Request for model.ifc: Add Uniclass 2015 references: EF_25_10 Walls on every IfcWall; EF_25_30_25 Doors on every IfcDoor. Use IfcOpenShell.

First a look at what the model holds.

```python
import ifcopenshell

model = ifcopenshell.open("model.ifc")
print(model.schema)
print("classifications:", [c.Name for c in model.by_type("IfcClassification")])
for ifc_class in ("IfcDoor", "IfcRoof", "IfcStair", "IfcWall", "IfcWindow"):
    print(ifc_class, len(model.by_type(ifc_class)))
```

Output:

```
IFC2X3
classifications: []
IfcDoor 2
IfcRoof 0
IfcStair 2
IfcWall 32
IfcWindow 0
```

```python
import ifcopenshell
import ifcopenshell.api.classification

model = ifcopenshell.open("model.ifc")

# IFC2X3 requires Source and Edition and has no link from the project to the system.
system = model.create_entity("IfcClassification", Source="NBS", Edition="2015", Name="Uniclass 2015")

codes = {
    "IfcWall": ("EF_25_10", "Walls"),
    "IfcDoor": ("EF_25_30_25", "Doors"),
}
for ifc_class, (code, name) in codes.items():
    products = model.by_type(ifc_class)
    ifcopenshell.api.classification.add_reference(
        model, products=products, classification=system, identification=code, name=name
    )
    print(code, len(products))

model.write("model_updated.ifc")
```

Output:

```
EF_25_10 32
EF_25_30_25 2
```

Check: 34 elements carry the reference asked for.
